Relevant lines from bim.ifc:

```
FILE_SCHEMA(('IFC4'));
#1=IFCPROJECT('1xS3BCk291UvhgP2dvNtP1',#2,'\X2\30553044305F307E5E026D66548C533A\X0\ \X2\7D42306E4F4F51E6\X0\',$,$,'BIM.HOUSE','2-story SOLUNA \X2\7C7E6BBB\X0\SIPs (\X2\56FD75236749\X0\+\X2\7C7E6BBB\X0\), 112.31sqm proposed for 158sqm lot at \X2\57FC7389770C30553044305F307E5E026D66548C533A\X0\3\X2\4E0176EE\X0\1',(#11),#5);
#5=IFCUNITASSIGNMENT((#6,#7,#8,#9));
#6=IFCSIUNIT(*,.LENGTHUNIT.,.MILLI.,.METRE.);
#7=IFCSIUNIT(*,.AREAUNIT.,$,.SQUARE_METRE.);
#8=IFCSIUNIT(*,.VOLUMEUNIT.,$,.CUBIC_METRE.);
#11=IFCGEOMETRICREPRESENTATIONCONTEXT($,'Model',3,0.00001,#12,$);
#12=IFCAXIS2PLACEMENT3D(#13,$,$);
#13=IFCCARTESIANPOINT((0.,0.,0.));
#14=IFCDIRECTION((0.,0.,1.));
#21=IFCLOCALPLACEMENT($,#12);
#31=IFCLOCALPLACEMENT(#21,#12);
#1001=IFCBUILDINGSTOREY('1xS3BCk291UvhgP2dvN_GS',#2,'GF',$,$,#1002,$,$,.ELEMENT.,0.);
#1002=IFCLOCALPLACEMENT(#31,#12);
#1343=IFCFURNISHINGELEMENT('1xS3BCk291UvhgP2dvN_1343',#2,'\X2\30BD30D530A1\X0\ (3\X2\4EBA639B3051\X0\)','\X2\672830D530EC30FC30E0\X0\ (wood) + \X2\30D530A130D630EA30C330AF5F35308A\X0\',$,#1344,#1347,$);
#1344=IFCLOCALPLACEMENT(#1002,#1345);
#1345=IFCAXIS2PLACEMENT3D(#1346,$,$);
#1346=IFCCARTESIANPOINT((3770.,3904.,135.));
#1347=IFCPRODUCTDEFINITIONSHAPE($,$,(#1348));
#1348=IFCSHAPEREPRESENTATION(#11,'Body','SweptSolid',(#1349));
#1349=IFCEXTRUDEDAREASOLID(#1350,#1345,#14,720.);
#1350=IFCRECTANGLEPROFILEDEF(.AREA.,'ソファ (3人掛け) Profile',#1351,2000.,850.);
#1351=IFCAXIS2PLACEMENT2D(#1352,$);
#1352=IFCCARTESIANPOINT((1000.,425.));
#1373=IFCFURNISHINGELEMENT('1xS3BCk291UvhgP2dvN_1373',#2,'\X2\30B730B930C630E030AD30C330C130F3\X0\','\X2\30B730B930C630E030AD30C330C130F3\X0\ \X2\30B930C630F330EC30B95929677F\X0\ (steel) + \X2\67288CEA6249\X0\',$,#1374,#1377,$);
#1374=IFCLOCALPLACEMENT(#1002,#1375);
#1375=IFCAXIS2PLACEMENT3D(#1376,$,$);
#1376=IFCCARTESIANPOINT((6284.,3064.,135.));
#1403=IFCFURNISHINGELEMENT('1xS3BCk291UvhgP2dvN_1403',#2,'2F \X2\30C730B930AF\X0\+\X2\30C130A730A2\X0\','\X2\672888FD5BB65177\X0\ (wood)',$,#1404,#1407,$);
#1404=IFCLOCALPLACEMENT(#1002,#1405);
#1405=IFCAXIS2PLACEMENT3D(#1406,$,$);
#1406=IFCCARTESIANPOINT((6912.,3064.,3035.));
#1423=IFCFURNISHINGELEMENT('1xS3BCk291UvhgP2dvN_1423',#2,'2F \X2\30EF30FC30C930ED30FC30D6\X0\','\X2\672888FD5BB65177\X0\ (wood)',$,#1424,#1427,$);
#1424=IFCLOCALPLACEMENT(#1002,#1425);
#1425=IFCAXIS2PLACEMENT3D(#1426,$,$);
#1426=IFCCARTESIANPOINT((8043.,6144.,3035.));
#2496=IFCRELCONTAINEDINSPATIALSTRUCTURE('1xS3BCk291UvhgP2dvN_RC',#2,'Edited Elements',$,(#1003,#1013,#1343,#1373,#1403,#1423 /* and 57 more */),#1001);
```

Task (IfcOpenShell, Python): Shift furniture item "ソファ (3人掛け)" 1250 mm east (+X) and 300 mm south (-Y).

```python
import ifcopenshell
import ifcopenshell.api.geometry
import ifcopenshell.util.placement
import ifcopenshell.util.unit

model = ifcopenshell.open("bim.ifc")
unit_scale = ifcopenshell.util.unit.calculate_unit_scale(model)

item = model.by_guid("1xS3BCk291UvhgP2dvN_1343")
matrix = ifcopenshell.util.placement.get_local_placement(item.ObjectPlacement)
matrix[0, 3] += 1.25 / unit_scale
matrix[1, 3] -= 0.3 / unit_scale
ifcopenshell.api.geometry.edit_object_placement(model, product=item, matrix=matrix, is_si=False)

print(ifcopenshell.util.placement.get_local_placement(item.ObjectPlacement).round(3) + 0.0)

model.write("bim_v2.ifc")
```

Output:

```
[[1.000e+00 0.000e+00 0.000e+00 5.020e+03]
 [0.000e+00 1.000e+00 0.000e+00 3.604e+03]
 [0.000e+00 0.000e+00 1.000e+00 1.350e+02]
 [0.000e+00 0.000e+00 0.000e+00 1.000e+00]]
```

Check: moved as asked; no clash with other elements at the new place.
